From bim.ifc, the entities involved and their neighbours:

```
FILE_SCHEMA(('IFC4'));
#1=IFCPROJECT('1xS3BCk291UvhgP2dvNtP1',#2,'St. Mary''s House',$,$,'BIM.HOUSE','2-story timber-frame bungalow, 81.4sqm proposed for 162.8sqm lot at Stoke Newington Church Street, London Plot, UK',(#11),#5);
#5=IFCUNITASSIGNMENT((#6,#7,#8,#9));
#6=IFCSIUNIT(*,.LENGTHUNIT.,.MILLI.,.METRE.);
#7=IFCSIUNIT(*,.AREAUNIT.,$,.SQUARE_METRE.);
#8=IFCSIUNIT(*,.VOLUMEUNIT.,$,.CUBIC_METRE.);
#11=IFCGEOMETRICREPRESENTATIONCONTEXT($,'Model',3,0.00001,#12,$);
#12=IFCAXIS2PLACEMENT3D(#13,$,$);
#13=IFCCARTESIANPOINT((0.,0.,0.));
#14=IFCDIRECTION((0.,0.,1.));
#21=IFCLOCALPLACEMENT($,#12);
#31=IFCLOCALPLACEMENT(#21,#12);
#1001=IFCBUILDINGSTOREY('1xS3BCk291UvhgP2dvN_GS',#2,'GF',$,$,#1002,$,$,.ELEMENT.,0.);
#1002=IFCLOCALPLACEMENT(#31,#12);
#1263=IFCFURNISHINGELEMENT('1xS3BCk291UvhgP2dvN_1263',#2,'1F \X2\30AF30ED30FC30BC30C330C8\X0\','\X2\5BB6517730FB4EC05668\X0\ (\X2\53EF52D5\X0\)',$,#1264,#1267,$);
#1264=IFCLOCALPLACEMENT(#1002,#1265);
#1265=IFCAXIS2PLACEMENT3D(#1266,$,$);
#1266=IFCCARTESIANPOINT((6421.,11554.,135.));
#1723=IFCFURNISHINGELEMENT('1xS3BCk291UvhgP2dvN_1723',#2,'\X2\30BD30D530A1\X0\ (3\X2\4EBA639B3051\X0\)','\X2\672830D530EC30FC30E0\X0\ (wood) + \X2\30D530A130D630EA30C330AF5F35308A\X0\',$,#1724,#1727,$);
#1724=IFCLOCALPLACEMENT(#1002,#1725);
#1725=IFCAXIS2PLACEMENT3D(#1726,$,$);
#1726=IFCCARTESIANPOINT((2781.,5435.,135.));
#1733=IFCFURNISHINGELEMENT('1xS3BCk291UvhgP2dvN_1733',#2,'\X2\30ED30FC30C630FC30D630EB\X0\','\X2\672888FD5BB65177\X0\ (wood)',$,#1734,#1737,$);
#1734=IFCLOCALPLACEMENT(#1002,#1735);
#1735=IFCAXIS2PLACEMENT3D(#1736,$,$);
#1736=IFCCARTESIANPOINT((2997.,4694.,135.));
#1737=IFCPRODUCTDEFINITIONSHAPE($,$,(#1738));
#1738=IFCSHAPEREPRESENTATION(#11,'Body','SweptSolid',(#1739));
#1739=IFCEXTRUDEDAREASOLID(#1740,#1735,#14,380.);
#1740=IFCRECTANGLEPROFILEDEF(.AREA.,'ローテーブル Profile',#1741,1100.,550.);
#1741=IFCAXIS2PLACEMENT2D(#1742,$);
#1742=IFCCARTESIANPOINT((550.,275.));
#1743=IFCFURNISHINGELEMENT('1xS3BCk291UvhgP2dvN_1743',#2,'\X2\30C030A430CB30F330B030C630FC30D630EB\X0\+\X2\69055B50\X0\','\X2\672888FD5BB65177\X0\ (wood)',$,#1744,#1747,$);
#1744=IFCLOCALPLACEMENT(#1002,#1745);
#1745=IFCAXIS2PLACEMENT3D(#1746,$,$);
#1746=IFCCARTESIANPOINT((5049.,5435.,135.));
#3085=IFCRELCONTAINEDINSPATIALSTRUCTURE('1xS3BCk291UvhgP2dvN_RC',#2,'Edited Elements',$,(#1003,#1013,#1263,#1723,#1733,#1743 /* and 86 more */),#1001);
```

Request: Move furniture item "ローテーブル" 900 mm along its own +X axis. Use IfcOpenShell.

```python
import ifcopenshell
import ifcopenshell.api.geometry
import ifcopenshell.util.placement
import ifcopenshell.util.unit

model = ifcopenshell.open("bim.ifc")
unit_scale = ifcopenshell.util.unit.calculate_unit_scale(model)

item = model.by_id(1733)
matrix = ifcopenshell.util.placement.get_local_placement(item.ObjectPlacement)
matrix[:3, 3] += matrix[:3, 0] * 0.9 / unit_scale
ifcopenshell.api.geometry.edit_object_placement(model, product=item, matrix=matrix, is_si=False)

print(ifcopenshell.util.placement.get_local_placement(item.ObjectPlacement).round(3) + 0.0)

model.write("bim_v2.ifc")
```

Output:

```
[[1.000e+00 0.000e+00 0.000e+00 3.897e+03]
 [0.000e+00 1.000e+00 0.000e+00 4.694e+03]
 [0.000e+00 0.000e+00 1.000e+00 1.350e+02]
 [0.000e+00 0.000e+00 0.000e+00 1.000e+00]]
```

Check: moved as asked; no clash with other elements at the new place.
